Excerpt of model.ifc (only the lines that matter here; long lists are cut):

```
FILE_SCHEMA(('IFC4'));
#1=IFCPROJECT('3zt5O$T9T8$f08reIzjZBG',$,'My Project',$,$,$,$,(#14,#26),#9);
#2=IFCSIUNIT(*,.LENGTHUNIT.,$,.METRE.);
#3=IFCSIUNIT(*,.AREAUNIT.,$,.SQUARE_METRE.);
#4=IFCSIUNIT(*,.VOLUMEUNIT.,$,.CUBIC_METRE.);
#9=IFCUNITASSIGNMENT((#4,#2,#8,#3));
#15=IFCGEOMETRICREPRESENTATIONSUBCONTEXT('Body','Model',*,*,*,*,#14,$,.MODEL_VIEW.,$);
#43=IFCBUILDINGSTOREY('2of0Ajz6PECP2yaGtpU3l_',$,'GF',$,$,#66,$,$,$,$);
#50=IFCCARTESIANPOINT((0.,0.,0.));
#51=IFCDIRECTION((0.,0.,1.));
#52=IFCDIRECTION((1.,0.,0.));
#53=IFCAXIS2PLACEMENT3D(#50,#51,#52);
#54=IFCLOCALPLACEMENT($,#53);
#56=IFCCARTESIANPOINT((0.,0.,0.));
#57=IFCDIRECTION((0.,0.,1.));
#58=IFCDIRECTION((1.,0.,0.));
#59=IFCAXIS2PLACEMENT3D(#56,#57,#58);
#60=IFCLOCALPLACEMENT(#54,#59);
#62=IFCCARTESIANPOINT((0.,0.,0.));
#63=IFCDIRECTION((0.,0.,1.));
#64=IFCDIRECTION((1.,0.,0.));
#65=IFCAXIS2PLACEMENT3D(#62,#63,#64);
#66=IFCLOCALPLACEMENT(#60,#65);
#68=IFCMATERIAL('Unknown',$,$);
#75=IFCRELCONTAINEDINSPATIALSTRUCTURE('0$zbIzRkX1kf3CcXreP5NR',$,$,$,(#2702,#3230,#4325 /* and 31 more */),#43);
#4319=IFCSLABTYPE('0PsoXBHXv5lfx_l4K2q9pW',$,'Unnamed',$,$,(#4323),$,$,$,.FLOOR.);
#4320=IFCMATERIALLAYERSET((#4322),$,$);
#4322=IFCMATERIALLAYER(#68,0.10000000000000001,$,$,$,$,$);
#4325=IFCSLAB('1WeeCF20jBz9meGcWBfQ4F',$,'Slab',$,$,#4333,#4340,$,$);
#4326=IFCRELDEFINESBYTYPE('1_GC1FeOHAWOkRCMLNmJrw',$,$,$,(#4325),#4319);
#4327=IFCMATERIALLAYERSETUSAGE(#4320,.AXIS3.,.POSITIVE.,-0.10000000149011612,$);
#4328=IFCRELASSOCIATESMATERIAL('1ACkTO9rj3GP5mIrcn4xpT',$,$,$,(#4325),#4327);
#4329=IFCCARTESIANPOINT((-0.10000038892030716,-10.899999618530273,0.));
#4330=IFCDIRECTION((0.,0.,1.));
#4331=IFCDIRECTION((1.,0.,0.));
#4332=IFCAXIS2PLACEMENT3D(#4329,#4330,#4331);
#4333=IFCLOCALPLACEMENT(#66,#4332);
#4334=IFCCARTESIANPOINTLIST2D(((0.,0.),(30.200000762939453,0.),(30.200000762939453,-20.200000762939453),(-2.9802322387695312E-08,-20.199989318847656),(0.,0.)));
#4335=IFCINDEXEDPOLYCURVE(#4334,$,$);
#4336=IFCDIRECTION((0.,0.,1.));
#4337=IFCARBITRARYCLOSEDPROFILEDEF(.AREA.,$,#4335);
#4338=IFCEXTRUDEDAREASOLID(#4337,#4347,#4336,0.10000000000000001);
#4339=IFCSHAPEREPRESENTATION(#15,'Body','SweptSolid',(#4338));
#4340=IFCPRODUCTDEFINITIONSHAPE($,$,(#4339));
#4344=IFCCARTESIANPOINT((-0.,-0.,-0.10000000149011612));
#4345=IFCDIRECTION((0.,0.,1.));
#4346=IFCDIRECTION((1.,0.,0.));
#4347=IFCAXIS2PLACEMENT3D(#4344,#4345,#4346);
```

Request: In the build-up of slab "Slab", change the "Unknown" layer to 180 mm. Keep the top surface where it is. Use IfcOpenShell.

```python
import ifcopenshell
import ifcopenshell.util.element
import ifcopenshell.util.representation
import ifcopenshell.util.unit

model = ifcopenshell.open("model.ifc")
unit_scale = ifcopenshell.util.unit.calculate_unit_scale(model)

layer_set = model.by_id(4320)
layer = next(l for l in layer_set.MaterialLayers if l.Material and l.Material.Name == "Unknown")
change = 0.18 / unit_scale - layer.LayerThickness
layer.LayerThickness += change

# Geometry does not follow the layer set by itself.
slabs = [e for e in ifcopenshell.util.element.get_elements_by_material(model, layer_set) if e.is_a("IfcSlab")]
for slab in sorted(slabs, key=lambda e: e.id()):
    body = ifcopenshell.util.representation.get_representation(slab, "Model", "Body")
    solid = body.Items[0]
    old_depth = solid.Depth
    solid.Depth += change
    # Extruded upwards: lower the start of the extrusion so the top stays.
    x, y, z = solid.Position.Location.Coordinates
    solid.Position.Location = model.createIfcCartesianPoint((x, y, z - change))
    print(slab.id(), f"{old_depth:g} -> {solid.Depth:g}")

# The layers are counted up from the underside, which has moved.
for usage in {ifcopenshell.util.element.get_material(slab) for slab in slabs}:
    usage.OffsetFromReferenceLine -= change

model.write("model_edited.ifc")
```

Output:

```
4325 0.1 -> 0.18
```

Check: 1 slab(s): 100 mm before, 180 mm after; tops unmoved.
